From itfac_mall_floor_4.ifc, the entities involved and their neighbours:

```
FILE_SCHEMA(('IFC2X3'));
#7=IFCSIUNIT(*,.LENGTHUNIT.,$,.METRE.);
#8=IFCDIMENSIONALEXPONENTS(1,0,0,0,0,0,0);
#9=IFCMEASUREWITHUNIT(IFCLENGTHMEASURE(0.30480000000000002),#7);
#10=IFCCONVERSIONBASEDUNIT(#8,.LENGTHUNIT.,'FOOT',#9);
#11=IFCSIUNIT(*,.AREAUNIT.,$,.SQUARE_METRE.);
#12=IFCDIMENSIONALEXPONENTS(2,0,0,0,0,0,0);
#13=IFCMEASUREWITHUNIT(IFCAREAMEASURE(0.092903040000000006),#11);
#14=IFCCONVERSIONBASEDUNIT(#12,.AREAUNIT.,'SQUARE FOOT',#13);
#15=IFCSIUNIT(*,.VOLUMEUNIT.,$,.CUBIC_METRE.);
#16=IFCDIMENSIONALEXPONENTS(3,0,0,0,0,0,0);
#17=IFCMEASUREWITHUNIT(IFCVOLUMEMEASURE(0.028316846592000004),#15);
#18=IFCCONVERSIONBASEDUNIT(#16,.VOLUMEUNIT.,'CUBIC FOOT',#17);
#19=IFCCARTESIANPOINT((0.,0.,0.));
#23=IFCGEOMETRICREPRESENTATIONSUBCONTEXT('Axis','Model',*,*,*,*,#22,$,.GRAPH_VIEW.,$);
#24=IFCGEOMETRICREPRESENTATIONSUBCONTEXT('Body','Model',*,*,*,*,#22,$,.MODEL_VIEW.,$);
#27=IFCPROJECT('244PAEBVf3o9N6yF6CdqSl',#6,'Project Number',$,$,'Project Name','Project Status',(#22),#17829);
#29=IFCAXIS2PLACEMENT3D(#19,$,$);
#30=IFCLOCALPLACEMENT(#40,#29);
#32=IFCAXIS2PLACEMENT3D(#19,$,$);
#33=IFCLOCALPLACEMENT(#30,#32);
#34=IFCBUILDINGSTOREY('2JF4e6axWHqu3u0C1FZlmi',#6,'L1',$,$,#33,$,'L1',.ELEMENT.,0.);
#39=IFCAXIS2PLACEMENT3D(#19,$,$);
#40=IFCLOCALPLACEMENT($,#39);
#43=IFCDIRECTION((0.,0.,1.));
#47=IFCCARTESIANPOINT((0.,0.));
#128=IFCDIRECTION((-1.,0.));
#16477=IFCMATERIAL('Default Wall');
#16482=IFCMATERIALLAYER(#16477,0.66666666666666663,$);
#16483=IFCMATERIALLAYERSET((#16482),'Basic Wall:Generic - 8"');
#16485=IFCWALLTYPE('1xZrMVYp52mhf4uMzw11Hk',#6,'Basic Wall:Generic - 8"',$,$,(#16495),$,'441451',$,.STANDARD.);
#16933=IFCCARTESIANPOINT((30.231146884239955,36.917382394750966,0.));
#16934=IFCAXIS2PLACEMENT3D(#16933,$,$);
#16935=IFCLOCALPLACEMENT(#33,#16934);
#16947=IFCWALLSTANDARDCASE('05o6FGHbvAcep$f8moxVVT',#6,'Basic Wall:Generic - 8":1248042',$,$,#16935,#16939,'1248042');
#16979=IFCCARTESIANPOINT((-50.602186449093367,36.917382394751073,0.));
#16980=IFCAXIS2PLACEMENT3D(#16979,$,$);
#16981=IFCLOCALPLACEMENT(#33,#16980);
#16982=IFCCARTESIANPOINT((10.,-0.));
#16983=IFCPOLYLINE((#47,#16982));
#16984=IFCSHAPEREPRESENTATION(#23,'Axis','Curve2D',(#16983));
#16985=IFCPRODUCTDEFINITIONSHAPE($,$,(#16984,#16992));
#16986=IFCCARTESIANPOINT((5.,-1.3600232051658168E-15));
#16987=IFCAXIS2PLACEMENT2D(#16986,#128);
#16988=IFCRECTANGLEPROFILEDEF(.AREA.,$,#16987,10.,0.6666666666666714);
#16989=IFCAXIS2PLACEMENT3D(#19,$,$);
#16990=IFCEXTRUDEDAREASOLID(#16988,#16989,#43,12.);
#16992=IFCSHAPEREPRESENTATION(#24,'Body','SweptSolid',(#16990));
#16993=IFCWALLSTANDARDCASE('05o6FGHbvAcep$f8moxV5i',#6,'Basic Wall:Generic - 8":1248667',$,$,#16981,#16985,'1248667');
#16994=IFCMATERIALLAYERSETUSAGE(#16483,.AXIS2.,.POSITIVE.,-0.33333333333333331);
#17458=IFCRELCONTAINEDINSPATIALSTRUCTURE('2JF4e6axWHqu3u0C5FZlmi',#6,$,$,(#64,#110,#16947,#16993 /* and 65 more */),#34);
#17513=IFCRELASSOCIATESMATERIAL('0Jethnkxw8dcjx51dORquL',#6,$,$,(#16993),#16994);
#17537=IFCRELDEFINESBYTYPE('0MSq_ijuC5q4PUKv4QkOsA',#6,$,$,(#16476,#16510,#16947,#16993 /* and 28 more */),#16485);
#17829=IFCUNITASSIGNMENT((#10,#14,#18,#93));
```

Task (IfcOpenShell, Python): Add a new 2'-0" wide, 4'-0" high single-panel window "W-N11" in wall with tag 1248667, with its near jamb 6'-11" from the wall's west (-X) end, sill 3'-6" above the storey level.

```python
import numpy as np
import ifcopenshell
import ifcopenshell.api.feature
import ifcopenshell.api.geometry
import ifcopenshell.api.root
import ifcopenshell.api.spatial
import ifcopenshell.api.type
import ifcopenshell.geom
import ifcopenshell.util.element
import ifcopenshell.util.placement
import ifcopenshell.util.representation
import ifcopenshell.util.shape
import ifcopenshell.util.unit

model = ifcopenshell.open("itfac_mall_floor_4.ifc")
unit_scale = ifcopenshell.util.unit.calculate_unit_scale(model)
settings = ifcopenshell.geom.settings()


def volume(element):
    """Net volume in cubic metres, openings subtracted."""
    shape = ifcopenshell.geom.create_shape(settings, element)
    return ifcopenshell.util.shape.get_volume(shape.geometry)


wall = model.by_guid("05o6FGHbvAcep$f8moxV5i")
storey = ifcopenshell.util.element.get_container(wall, ifc_class="IfcBuildingStorey")
context = ifcopenshell.util.representation.get_context(model, "Model", "Body", "MODEL_VIEW")
before = volume(wall)

width, height, from_end, sill = 0.6096, 1.2192, 2.1082, 1.0668  # metres

# The wall runs along its own X axis, and the end named is its -X end.
wall_shape = ifcopenshell.geom.create_shape(settings, wall)
x, y, z = ifcopenshell.util.shape.get_vertices(wall_shape.geometry).T
start = x.min() + from_end
face, thickness = float(y.min()), float(y.max() - y.min())
wall_matrix = ifcopenshell.util.placement.get_local_placement(wall.ObjectPlacement)
level = ifcopenshell.util.placement.get_local_placement(storey.ObjectPlacement)[2, 3]


def in_wall(x, y):
    """Placement at x, y metres in the wall's axes, at sill height."""
    matrix = wall_matrix.copy()
    matrix[:, 3] = wall_matrix @ np.array([x / unit_scale, y / unit_scale, 0.0, 1.0])
    matrix[2, 3] = level + sill / unit_scale
    return matrix


# Opening: a box that overshoots both wall faces by 50 mm.
opening = ifcopenshell.api.root.create_entity(model, ifc_class="IfcOpeningElement")
box = ifcopenshell.api.geometry.add_wall_representation(
    model, context=context, length=width, height=height, thickness=thickness + 0.1
)
ifcopenshell.api.geometry.assign_representation(model, product=opening, representation=box)
ifcopenshell.api.geometry.edit_object_placement(model, product=opening, matrix=in_wall(start, face - 0.05), is_si=False)
ifcopenshell.api.feature.add_feature(model, feature=opening, element=wall)

window = ifcopenshell.api.root.create_entity(model, ifc_class="IfcWindow", name="W-N11")
window.OverallWidth, window.OverallHeight = width / unit_scale, height / unit_scale
body = ifcopenshell.api.geometry.add_window_representation(
    model,
    context=context,
    overall_width=window.OverallWidth,
    overall_height=window.OverallHeight,
    partition_type="SINGLE_PANEL",
)
ifcopenshell.api.geometry.assign_representation(model, product=window, representation=body)
ifcopenshell.api.spatial.assign_container(model, products=[window], relating_structure=storey)
fills = ifcopenshell.api.feature.add_filling(model, opening=opening, element=window)
fills.OwnerHistory = window.OwnerHistory  # required in IFC2X3

# IFC2X3 keeps the operation on the window style.
style = ifcopenshell.api.root.create_entity(model, ifc_class="IfcWindowStyle", name="W-N11")
style.OperationType, style.ConstructionType = "SINGLE_PANEL", "NOTDEFINED"
style.ParameterTakesPrecedence = style.Sizeable = False
ifcopenshell.api.type.assign_type(model, related_objects=[window], relating_type=style)

# Centre the window in the wall's thickness.
ifcopenshell.api.geometry.edit_object_placement(model, product=window, matrix=in_wall(start, face), is_si=False)
window_shape = ifcopenshell.geom.create_shape(settings, window)
depth = ifcopenshell.util.shape.get_vertices(window_shape.geometry)[:, 1]
offset = face + thickness / 2 - (depth.min() + depth.max()) / 2
ifcopenshell.api.geometry.edit_object_placement(model, product=window, matrix=in_wall(start, offset), is_si=False)

after = volume(wall)

print(f"wall volume {before:.3f} -> {after:.3f} m3")

model.write("itfac_mall_floor_4_edited.ifc")
```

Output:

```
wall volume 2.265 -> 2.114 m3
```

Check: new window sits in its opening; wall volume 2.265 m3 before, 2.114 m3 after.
